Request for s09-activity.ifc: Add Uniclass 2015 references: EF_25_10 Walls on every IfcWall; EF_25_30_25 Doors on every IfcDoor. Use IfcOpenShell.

First a look at what the model holds.

```python
import ifcopenshell

model = ifcopenshell.open("s09-activity.ifc")
print(model.schema)
print("classifications:", [c.Name for c in model.by_type("IfcClassification")])
for ifc_class in ("IfcDoor", "IfcRoof", "IfcStair", "IfcWall", "IfcWindow"):
    print(ifc_class, len(model.by_type(ifc_class)))
```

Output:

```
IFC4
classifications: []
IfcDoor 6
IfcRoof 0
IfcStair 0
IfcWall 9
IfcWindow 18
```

```python
import ifcopenshell
import ifcopenshell.api.classification

model = ifcopenshell.open("s09-activity.ifc")

system = ifcopenshell.api.classification.add_classification(model, classification="Uniclass 2015")

codes = {
    "IfcWall": ("EF_25_10", "Walls"),
    "IfcDoor": ("EF_25_30_25", "Doors"),
}
for ifc_class, (code, name) in codes.items():
    products = model.by_type(ifc_class)
    ifcopenshell.api.classification.add_reference(
        model, products=products, classification=system, identification=code, name=name
    )
    print(code, len(products))

model.write("s09-activity-out.ifc")
```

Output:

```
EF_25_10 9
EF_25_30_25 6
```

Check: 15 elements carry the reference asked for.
